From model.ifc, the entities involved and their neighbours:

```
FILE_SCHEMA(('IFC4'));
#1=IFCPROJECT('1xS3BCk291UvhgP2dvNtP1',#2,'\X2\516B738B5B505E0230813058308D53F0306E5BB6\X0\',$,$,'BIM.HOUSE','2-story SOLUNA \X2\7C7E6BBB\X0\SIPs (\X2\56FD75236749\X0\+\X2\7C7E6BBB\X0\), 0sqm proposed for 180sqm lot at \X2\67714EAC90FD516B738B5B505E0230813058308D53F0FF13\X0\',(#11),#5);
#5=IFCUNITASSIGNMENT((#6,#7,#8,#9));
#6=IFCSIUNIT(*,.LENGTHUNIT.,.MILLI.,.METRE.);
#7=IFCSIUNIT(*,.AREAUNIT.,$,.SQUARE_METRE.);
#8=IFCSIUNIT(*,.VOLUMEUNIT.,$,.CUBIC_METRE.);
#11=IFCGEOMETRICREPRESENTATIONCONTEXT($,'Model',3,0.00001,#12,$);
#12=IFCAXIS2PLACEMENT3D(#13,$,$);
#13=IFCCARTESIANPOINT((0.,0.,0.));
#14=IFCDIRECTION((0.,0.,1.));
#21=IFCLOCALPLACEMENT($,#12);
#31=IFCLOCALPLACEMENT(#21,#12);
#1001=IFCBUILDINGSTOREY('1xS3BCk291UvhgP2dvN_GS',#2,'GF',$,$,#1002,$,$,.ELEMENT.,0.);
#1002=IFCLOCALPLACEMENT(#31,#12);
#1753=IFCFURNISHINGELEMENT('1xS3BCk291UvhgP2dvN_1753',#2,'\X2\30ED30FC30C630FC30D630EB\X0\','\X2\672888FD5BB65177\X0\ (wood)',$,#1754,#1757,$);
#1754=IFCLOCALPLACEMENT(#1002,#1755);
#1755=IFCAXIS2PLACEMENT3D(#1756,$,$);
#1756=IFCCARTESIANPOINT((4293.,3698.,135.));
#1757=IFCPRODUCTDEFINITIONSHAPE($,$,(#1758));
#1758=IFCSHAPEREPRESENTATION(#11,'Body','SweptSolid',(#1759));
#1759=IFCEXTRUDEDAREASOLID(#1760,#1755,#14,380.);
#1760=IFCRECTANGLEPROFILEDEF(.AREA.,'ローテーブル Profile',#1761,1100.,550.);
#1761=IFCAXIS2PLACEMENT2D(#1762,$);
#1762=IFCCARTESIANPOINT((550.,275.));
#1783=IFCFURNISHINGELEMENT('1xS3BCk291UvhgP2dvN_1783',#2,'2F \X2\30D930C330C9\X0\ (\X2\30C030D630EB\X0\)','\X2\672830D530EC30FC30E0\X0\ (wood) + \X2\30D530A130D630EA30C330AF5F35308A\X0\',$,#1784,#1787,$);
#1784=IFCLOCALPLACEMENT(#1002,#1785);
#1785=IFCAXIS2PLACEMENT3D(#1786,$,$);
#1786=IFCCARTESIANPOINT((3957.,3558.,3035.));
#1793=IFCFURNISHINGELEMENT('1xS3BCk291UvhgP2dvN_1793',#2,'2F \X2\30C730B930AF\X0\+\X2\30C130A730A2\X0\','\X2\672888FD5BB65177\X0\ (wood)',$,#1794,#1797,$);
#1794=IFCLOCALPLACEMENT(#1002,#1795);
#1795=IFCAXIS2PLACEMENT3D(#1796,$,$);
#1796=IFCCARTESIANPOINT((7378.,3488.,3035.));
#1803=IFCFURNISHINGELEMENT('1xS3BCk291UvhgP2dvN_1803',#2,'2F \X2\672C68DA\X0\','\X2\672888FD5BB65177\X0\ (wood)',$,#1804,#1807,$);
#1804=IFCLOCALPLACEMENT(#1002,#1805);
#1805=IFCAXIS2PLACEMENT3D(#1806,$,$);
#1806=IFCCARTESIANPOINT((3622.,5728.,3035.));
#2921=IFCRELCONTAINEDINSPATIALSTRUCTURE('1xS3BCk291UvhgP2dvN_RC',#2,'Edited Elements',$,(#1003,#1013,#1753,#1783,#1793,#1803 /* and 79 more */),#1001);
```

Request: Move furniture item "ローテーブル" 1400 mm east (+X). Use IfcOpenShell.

```python
import ifcopenshell
import ifcopenshell.api.geometry
import ifcopenshell.util.placement

model = ifcopenshell.open("model.ifc")

item = model.by_id(1753)
matrix = ifcopenshell.util.placement.get_local_placement(item.ObjectPlacement)
matrix[0, 3] += 1400.0
ifcopenshell.api.geometry.edit_object_placement(model, product=item, matrix=matrix, is_si=False)

print(ifcopenshell.util.placement.get_local_placement(item.ObjectPlacement).round(3) + 0.0)

model.write("model_updated.ifc")
```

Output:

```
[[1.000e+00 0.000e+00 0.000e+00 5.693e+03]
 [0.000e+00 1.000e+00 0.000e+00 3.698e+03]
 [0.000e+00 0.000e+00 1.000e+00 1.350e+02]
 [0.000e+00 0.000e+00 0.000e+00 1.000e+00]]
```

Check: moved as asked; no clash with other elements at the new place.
